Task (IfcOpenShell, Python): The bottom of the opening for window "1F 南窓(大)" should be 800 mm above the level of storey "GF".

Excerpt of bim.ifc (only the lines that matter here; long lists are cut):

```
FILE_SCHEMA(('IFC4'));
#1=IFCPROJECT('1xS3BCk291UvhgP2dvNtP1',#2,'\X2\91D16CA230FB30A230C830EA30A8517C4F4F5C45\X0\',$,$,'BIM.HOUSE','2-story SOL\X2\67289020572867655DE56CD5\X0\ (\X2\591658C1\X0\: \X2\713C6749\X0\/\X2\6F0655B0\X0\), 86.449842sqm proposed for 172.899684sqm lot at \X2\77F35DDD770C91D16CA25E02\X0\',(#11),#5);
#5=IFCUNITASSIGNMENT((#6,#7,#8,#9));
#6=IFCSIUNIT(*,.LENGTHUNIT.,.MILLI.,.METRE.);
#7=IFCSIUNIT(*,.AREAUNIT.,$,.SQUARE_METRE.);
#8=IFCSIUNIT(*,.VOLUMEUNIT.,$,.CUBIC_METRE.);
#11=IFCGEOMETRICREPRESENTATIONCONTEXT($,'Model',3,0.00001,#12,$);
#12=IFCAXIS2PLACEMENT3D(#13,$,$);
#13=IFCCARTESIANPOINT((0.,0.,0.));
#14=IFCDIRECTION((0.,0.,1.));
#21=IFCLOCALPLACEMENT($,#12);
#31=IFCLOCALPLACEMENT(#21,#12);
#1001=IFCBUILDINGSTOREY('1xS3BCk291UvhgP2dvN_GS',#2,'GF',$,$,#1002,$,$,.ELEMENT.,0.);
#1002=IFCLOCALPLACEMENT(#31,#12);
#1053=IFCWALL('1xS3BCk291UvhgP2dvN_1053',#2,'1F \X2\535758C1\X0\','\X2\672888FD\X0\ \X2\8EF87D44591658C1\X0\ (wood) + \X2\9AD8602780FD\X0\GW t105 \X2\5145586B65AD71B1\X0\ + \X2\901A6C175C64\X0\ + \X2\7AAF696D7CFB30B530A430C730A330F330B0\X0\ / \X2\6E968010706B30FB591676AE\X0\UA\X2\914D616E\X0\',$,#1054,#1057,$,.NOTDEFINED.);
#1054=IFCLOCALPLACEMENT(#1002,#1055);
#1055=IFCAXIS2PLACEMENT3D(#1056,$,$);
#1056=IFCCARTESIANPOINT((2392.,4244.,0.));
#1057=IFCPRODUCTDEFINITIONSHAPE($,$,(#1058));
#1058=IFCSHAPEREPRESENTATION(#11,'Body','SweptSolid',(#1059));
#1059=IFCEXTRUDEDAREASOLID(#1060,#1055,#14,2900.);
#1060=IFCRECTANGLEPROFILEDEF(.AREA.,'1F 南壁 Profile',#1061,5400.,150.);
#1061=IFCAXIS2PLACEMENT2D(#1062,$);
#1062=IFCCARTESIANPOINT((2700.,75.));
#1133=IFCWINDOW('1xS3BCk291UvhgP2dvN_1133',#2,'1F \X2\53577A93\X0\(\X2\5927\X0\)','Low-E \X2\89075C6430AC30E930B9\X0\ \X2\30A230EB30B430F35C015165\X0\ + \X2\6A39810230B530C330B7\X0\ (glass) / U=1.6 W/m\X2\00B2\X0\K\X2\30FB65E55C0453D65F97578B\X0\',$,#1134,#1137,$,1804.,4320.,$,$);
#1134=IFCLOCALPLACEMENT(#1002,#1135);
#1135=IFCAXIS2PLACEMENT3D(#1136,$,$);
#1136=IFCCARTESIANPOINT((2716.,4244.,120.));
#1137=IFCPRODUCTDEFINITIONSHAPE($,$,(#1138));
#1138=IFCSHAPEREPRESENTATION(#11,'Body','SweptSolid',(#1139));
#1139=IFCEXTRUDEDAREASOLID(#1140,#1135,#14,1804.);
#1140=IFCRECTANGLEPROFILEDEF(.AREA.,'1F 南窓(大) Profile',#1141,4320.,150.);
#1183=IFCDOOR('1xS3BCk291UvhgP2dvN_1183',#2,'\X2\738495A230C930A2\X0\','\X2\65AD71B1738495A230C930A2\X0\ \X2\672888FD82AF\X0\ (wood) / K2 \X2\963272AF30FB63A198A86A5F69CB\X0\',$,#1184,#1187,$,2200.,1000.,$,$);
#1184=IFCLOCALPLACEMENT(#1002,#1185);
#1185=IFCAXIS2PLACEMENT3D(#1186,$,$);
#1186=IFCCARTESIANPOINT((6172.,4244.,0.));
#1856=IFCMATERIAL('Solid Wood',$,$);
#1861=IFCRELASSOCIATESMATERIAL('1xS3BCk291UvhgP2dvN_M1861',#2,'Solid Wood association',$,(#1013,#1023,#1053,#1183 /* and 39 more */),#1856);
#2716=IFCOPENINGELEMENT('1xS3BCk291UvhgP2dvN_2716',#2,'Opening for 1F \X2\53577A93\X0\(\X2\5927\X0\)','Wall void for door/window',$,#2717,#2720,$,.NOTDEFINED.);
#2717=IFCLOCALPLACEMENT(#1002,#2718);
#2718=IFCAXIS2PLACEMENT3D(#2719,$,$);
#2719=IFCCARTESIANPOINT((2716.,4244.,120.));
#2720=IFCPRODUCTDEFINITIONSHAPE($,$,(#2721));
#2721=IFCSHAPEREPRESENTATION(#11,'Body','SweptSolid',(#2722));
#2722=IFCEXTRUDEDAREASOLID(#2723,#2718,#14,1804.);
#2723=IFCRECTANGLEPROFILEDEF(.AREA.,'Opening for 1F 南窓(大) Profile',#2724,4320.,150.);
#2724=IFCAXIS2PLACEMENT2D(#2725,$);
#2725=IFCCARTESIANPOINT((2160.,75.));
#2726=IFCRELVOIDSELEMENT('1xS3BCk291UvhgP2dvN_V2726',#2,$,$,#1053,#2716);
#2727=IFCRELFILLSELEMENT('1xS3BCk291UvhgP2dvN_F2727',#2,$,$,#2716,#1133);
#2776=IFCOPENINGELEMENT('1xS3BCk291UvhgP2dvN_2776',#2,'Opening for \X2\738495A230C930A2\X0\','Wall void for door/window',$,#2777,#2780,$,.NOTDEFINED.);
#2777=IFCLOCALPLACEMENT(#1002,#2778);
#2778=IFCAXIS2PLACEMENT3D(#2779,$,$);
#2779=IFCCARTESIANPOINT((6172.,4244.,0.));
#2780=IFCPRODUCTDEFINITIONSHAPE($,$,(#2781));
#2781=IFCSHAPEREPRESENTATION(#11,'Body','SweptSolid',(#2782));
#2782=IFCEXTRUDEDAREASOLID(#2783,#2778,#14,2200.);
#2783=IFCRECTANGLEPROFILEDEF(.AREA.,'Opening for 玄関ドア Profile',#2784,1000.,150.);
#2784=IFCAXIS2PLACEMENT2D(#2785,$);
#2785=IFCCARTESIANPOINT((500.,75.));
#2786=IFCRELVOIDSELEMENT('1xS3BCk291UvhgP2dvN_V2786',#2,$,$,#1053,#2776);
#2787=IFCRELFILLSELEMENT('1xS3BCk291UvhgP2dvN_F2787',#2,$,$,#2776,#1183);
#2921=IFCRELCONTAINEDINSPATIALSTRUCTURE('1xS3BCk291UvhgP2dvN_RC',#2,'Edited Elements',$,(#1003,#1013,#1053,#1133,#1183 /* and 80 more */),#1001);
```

```python
import numpy as np
import ifcopenshell
import ifcopenshell.api.geometry
import ifcopenshell.geom
import ifcopenshell.util.element
import ifcopenshell.util.placement
import ifcopenshell.util.shape
import ifcopenshell.util.unit

model = ifcopenshell.open("bim.ifc")
unit_scale = ifcopenshell.util.unit.calculate_unit_scale(model)

window = model.by_guid("1xS3BCk291UvhgP2dvN_1133")
opening = window.FillsVoids[0].RelatingOpeningElement
storey = ifcopenshell.util.element.get_container(window, ifc_class="IfcBuildingStorey")
level = ifcopenshell.util.placement.get_local_placement(storey.ObjectPlacement)[2, 3]

# The opening's origin need not be at the sill, so measure its lowest point.
shape = ifcopenshell.geom.create_shape(ifcopenshell.geom.settings(), opening)
bottom = ifcopenshell.util.shape.get_shape_bottom_elevation(shape, shape.geometry) / unit_scale
dz = level + 0.8 / unit_scale - bottom

shift = np.array([0.0, 0.0, dz])
# The window is not placed relative to its opening, so move both.
for product in (opening, window):
    matrix = ifcopenshell.util.placement.get_local_placement(product.ObjectPlacement)
    matrix[:3, 3] += shift
    ifcopenshell.api.geometry.edit_object_placement(model, product=product, matrix=matrix, is_si=False)

print(f"moved by {dz * unit_scale:+.3f} m")

model.write("bim-out.ifc")
```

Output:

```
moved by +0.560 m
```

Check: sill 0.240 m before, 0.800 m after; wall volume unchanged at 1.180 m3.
